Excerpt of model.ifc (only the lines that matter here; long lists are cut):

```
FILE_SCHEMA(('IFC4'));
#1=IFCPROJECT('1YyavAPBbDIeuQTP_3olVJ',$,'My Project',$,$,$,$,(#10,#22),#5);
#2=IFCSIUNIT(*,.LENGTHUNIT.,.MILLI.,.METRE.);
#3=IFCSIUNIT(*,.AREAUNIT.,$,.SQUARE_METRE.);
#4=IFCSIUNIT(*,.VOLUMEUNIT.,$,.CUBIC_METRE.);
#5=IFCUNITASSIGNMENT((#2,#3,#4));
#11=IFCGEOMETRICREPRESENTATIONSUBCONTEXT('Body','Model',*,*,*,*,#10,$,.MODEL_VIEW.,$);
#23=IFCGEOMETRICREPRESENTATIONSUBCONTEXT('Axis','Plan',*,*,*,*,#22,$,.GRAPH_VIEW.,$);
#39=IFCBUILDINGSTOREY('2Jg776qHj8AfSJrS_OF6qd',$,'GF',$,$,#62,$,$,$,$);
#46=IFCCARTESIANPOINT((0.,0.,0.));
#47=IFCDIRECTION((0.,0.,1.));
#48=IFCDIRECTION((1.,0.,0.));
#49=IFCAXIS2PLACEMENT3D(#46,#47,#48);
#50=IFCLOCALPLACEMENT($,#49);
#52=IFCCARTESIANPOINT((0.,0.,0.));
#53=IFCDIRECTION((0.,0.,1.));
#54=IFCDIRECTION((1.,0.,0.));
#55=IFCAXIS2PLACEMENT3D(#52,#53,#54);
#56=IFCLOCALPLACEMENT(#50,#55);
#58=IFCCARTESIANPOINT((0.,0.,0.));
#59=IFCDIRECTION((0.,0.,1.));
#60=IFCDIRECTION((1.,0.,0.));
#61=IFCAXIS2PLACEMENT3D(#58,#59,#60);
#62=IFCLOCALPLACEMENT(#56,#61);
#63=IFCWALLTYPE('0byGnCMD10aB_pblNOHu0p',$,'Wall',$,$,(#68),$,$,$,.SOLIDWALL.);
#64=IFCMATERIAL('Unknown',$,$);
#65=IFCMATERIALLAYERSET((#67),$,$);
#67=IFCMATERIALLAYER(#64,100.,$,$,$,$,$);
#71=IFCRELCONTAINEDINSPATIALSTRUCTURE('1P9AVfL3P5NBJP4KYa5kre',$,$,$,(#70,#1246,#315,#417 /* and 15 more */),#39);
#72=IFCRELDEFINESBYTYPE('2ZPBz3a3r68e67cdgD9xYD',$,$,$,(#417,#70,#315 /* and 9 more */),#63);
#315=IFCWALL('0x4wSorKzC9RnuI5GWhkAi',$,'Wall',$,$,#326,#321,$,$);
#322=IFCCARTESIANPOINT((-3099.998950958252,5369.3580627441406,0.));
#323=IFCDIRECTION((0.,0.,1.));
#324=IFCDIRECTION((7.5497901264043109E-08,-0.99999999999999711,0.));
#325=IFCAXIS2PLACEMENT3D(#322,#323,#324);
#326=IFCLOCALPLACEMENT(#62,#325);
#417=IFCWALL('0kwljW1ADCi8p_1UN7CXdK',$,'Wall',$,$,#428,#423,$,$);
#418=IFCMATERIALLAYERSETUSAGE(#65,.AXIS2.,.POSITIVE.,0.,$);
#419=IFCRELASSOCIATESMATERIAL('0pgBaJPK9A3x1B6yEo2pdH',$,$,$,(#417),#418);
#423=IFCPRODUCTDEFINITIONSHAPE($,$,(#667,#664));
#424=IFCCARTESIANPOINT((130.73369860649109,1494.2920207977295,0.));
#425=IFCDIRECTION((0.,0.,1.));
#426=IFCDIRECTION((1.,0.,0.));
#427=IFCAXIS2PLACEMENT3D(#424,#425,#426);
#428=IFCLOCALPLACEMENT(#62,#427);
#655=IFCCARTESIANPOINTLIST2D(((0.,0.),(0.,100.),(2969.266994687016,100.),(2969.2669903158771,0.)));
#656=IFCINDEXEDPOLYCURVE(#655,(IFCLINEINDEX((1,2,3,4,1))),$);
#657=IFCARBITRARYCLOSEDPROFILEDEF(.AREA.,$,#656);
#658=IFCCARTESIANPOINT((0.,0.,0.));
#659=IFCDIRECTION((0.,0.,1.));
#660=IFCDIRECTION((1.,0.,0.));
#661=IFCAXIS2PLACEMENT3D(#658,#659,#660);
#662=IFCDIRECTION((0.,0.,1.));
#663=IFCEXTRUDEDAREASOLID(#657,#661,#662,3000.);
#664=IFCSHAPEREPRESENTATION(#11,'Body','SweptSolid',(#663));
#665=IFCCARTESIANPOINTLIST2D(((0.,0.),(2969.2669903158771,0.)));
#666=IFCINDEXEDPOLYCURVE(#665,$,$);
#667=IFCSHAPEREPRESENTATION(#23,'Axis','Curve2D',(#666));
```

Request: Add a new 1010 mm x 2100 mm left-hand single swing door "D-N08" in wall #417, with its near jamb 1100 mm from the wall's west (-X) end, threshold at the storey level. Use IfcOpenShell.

```python
import numpy as np
import ifcopenshell
import ifcopenshell.api.feature
import ifcopenshell.api.geometry
import ifcopenshell.api.root
import ifcopenshell.api.spatial
import ifcopenshell.geom
import ifcopenshell.util.element
import ifcopenshell.util.placement
import ifcopenshell.util.representation
import ifcopenshell.util.shape
import ifcopenshell.util.unit

model = ifcopenshell.open("model.ifc")
unit_scale = ifcopenshell.util.unit.calculate_unit_scale(model)
settings = ifcopenshell.geom.settings()


def volume(element):
    """Net volume in cubic metres, openings subtracted."""
    shape = ifcopenshell.geom.create_shape(settings, element)
    return ifcopenshell.util.shape.get_volume(shape.geometry)


wall = model.by_guid("0kwljW1ADCi8p_1UN7CXdK")
storey = ifcopenshell.util.element.get_container(wall, ifc_class="IfcBuildingStorey")
context = ifcopenshell.util.representation.get_context(model, "Model", "Body", "MODEL_VIEW")
before = volume(wall)

width, height, from_end, sill = 1.01, 2.1, 1.1, 0.0  # metres

# The wall runs along its own X axis, and the end named is its -X end.
wall_shape = ifcopenshell.geom.create_shape(settings, wall)
x, y, z = ifcopenshell.util.shape.get_vertices(wall_shape.geometry).T
start = x.min() + from_end
face, thickness = float(y.min()), float(y.max() - y.min())
wall_matrix = ifcopenshell.util.placement.get_local_placement(wall.ObjectPlacement)
level = ifcopenshell.util.placement.get_local_placement(storey.ObjectPlacement)[2, 3]


def in_wall(x, y):
    """Placement at x, y metres in the wall's axes, at sill height."""
    matrix = wall_matrix.copy()
    matrix[:, 3] = wall_matrix @ np.array([x / unit_scale, y / unit_scale, 0.0, 1.0])
    matrix[2, 3] = level + sill / unit_scale
    return matrix


# Opening: a box that overshoots both wall faces by 50 mm.
opening = ifcopenshell.api.root.create_entity(model, ifc_class="IfcOpeningElement", predefined_type="OPENING")
box = ifcopenshell.api.geometry.add_wall_representation(
    model, context=context, length=width, height=height, thickness=thickness + 0.1
)
ifcopenshell.api.geometry.assign_representation(model, product=opening, representation=box)
ifcopenshell.api.geometry.edit_object_placement(model, product=opening, matrix=in_wall(start, face - 0.05), is_si=False)
ifcopenshell.api.feature.add_feature(model, feature=opening, element=wall)

door = ifcopenshell.api.root.create_entity(model, ifc_class="IfcDoor", name="D-N08", predefined_type="DOOR")
door.OverallWidth, door.OverallHeight = width / unit_scale, height / unit_scale
door.OperationType = "SINGLE_SWING_LEFT"
body = ifcopenshell.api.geometry.add_door_representation(
    model,
    context=context,
    overall_width=door.OverallWidth,
    overall_height=door.OverallHeight,
    operation_type="SINGLE_SWING_LEFT",
    lining_properties={"LiningDepth": thickness / unit_scale, "ThresholdDepth": thickness / unit_scale},
)
ifcopenshell.api.geometry.assign_representation(model, product=door, representation=body)
ifcopenshell.api.spatial.assign_container(model, products=[door], relating_structure=storey)
ifcopenshell.api.feature.add_filling(model, opening=opening, element=door)

# The lining spans the wall, so the door starts at the wall face.
ifcopenshell.api.geometry.edit_object_placement(model, product=door, matrix=in_wall(start, face), is_si=False)

after = volume(wall)

print(f"wall volume {before:.3f} -> {after:.3f} m3")

model.write("model_edited.ifc")
```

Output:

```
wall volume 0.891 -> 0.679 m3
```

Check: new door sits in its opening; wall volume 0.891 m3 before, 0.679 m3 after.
